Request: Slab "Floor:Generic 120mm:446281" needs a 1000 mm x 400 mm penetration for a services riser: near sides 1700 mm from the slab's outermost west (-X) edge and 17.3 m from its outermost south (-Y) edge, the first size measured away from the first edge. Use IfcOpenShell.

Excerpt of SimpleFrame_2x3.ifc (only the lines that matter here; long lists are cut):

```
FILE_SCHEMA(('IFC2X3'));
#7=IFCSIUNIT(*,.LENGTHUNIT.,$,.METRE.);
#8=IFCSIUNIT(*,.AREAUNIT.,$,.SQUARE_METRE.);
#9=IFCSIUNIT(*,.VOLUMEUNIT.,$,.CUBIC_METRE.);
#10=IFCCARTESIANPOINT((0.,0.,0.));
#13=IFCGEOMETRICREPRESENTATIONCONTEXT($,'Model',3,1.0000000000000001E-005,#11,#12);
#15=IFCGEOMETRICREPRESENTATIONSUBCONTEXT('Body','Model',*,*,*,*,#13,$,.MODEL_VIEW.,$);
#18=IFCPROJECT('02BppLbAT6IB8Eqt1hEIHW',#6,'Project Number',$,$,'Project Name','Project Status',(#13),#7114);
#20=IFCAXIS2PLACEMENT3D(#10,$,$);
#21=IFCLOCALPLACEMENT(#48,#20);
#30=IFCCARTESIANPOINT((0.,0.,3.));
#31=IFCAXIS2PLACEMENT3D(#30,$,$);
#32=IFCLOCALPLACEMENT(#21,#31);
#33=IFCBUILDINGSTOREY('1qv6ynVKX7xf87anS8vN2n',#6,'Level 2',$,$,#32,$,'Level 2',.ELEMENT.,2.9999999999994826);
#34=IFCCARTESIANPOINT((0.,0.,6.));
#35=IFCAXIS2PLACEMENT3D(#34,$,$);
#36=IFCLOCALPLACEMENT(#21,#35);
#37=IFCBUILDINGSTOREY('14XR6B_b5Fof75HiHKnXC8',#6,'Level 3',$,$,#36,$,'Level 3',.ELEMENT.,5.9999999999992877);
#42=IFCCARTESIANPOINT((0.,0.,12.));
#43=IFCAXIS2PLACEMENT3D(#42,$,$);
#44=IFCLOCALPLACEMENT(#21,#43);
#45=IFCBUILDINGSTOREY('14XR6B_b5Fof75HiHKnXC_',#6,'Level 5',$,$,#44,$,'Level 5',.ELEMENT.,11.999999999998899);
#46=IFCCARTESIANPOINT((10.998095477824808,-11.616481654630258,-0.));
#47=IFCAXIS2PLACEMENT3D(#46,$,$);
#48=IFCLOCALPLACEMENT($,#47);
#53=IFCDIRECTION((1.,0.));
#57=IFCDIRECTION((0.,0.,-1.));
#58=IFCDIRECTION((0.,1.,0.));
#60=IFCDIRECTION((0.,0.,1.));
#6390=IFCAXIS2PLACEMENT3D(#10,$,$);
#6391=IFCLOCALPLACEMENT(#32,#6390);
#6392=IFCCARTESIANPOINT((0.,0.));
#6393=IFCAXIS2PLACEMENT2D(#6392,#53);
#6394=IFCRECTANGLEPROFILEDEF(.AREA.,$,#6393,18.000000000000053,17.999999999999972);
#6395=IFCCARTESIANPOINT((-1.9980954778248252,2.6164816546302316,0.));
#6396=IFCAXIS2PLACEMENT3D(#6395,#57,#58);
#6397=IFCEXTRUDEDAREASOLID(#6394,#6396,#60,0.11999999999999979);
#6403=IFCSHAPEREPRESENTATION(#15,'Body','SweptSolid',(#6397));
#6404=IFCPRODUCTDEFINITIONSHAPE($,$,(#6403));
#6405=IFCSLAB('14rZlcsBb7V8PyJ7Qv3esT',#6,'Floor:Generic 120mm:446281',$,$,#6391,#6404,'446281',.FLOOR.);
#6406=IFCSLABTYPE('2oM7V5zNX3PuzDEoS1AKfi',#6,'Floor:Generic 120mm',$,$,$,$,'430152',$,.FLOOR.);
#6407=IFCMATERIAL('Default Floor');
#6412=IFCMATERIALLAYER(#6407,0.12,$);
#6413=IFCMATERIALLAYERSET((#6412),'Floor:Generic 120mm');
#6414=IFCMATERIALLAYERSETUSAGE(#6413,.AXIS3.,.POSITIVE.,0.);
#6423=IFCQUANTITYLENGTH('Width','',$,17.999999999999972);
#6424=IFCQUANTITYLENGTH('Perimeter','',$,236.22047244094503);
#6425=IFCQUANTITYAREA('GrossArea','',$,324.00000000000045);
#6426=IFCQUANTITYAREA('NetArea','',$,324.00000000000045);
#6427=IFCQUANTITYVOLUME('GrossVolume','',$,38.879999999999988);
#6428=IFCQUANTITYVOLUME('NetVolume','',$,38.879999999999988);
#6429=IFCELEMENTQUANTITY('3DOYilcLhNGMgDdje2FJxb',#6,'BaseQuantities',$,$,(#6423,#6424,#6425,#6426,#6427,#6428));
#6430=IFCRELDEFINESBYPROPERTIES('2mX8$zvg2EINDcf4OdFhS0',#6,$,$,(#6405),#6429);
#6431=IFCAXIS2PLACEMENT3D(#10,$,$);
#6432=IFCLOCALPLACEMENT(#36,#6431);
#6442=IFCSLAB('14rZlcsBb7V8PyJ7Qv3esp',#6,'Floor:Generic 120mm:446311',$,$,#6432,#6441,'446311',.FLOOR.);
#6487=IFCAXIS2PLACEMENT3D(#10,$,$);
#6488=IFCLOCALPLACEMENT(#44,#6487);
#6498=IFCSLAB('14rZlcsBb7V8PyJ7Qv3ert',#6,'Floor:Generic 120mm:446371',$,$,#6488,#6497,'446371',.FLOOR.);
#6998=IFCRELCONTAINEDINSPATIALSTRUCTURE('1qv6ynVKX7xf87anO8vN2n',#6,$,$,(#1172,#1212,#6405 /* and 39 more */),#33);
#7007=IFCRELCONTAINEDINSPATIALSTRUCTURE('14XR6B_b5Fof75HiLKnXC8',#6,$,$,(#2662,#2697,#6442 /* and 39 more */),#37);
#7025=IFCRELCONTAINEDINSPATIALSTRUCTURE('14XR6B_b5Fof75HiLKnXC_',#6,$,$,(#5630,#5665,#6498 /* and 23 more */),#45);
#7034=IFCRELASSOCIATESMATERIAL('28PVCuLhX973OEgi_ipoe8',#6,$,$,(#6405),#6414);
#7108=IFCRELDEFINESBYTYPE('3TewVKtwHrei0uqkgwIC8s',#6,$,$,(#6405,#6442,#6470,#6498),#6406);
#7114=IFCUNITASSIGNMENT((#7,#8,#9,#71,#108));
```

```python
import numpy as np
import ifcopenshell
import ifcopenshell.api.feature
import ifcopenshell.api.geometry
import ifcopenshell.api.pset
import ifcopenshell.api.root
import ifcopenshell.geom
import ifcopenshell.util.element
import ifcopenshell.util.placement
import ifcopenshell.util.representation
import ifcopenshell.util.shape
import ifcopenshell.util.unit

model = ifcopenshell.open("SimpleFrame_2x3.ifc")
unit_scale = ifcopenshell.util.unit.calculate_unit_scale(model)
area_scale = ifcopenshell.util.unit.calculate_unit_scale(model, "AREAUNIT")
volume_scale = ifcopenshell.util.unit.calculate_unit_scale(model, "VOLUMEUNIT")
settings = ifcopenshell.geom.settings()


def volume(element):
    """Net volume in cubic metres, openings subtracted."""
    shape = ifcopenshell.geom.create_shape(settings, element)
    return ifcopenshell.util.shape.get_volume(shape.geometry)


slab = model.by_id(6405)
before = volume(slab)

# Extent in the slab's own axes, in metres. The edges named are its -X and -Y sides.
slab_shape = ifcopenshell.geom.create_shape(settings, slab)
vertices = ifcopenshell.util.shape.get_vertices(slab_shape.geometry)
x_min, y_min, bottom = vertices.min(axis=0)
top = vertices[:, 2].max()

opening = ifcopenshell.api.root.create_entity(model, ifc_class="IfcOpeningElement", name="Services riser opening")
context = ifcopenshell.util.representation.get_context(model, "Model", "Body", "MODEL_VIEW")
width, depth = 1, 0.4
outline = [(0.0, 0.0), (width, 0.0), (width, depth), (0.0, depth), (0.0, 0.0)]
# Overshoot both faces by 50 mm so the cut is clean.
shape = ifcopenshell.api.geometry.add_slab_representation(
    model, context=context, depth=top - bottom + 0.1, polyline=outline
)
ifcopenshell.api.geometry.assign_representation(model, product=opening, representation=shape)

matrix = ifcopenshell.util.placement.get_local_placement(slab.ObjectPlacement)
matrix[:, 3] = matrix @ np.append(np.array([x_min + 1.7, y_min + 17.3, bottom - 0.05]) / unit_scale, 1.0)
ifcopenshell.api.geometry.edit_object_placement(model, product=opening, matrix=matrix, is_si=False)
ifcopenshell.api.feature.add_feature(model, feature=opening, element=slab)

after = volume(slab)

# Update the slab's stored quantities.
qto = model.by_id(ifcopenshell.util.element.get_pset(slab, "BaseQuantities", should_inherit=False)["id"])
ifcopenshell.api.pset.edit_qto(model, qto=qto, properties={
    "NetArea": after / (top - bottom) / area_scale,
    "NetVolume": after / volume_scale,
})

print(f"slab volume {before:.3f} -> {after:.3f} m3")

model.write("SimpleFrame_2x3-out.ifc")
```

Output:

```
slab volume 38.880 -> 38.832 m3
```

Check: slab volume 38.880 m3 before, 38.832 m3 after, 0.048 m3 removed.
